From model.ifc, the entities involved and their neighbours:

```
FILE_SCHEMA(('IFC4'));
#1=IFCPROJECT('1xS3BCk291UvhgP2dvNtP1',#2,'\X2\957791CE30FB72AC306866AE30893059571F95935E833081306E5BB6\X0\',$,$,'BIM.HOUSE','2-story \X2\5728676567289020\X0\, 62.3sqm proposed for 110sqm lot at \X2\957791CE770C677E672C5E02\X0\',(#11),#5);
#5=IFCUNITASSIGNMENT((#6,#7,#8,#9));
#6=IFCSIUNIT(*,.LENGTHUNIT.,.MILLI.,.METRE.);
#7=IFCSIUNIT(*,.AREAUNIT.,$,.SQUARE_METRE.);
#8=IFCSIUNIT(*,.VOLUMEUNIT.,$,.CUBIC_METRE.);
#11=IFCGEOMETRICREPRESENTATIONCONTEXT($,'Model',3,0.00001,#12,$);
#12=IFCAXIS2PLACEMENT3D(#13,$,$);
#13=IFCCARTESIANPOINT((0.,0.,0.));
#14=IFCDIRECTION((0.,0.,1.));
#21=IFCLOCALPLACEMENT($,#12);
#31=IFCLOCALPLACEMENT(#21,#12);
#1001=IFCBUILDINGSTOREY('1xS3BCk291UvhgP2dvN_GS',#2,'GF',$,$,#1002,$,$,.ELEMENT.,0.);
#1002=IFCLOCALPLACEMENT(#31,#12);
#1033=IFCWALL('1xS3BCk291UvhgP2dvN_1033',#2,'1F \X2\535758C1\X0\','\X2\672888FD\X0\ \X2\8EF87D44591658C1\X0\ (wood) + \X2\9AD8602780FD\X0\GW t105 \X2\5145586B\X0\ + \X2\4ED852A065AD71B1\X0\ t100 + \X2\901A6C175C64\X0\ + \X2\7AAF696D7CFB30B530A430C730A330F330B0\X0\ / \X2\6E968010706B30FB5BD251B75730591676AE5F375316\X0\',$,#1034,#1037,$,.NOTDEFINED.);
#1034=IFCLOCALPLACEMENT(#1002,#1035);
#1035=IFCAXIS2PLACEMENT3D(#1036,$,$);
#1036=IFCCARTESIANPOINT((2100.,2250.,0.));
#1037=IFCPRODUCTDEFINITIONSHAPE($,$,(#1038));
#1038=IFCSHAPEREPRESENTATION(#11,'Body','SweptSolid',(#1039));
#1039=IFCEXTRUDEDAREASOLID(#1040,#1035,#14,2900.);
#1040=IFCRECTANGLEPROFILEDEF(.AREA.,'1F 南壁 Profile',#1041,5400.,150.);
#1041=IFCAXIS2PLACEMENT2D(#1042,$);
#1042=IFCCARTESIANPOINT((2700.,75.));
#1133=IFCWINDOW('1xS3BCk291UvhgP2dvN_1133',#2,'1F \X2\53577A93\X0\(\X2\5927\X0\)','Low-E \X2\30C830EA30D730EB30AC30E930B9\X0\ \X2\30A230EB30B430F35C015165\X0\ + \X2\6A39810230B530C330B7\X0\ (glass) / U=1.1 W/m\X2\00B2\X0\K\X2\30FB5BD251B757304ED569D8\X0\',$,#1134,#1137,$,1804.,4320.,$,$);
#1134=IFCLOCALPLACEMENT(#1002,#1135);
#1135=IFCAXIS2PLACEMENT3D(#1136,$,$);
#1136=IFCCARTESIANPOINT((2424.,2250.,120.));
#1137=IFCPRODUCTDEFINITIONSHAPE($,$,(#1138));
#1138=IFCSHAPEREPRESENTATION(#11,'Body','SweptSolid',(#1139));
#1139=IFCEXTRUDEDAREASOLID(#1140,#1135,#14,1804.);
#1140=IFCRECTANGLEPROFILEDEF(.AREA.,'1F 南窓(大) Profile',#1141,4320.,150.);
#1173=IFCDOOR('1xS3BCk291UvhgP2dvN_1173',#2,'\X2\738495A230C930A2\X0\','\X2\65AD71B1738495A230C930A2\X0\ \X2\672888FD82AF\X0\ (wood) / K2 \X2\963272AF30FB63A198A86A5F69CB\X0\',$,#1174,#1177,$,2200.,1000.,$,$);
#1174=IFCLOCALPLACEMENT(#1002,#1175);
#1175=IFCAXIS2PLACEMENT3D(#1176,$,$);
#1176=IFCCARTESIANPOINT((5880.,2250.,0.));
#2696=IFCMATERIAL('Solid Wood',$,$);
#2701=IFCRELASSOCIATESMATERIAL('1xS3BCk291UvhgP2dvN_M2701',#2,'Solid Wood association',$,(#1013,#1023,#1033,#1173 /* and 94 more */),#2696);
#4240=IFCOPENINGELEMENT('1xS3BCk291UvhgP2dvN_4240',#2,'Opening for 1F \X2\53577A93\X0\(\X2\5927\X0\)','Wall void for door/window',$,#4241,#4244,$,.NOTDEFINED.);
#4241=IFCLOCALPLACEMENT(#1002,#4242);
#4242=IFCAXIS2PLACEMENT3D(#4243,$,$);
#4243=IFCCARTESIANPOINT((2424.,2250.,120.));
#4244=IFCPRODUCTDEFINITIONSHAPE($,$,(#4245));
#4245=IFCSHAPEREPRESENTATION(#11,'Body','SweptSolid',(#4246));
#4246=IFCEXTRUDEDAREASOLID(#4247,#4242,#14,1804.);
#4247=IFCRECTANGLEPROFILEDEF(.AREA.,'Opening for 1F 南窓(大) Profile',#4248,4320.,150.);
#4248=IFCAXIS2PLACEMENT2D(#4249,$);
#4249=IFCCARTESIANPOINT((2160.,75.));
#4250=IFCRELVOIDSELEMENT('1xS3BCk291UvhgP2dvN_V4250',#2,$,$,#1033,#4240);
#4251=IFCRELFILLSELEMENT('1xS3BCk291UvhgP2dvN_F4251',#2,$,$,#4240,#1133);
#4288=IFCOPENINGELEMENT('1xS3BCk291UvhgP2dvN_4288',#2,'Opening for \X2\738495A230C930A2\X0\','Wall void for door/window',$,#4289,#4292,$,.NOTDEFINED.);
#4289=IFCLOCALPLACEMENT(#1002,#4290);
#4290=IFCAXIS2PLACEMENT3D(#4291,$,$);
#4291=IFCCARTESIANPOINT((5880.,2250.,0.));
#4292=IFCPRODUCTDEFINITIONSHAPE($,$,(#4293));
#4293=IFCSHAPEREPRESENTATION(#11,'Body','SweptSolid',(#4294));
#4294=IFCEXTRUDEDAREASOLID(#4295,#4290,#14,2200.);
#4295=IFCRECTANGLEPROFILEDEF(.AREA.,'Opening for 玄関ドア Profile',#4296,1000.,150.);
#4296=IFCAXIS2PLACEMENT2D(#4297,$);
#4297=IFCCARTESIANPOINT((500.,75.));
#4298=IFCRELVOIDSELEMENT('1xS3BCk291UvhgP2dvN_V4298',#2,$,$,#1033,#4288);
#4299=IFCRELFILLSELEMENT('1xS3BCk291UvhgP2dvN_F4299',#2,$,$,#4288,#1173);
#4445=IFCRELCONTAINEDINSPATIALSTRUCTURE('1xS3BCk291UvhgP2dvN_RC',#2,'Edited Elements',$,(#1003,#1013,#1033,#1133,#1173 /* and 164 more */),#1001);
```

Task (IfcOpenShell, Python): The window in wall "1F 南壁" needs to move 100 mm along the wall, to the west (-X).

```python
import ifcopenshell
import ifcopenshell.api.geometry
import ifcopenshell.util.placement
import ifcopenshell.util.unit

model = ifcopenshell.open("model.ifc")
unit_scale = ifcopenshell.util.unit.calculate_unit_scale(model)

window = model.by_guid("1xS3BCk291UvhgP2dvN_1133")
opening = window.FillsVoids[0].RelatingOpeningElement
wall = opening.VoidsElements[0].RelatingBuildingElement

wall_matrix = ifcopenshell.util.placement.get_local_placement(wall.ObjectPlacement)
shift = wall_matrix[:3, 0] * -0.1 / unit_scale
before = ifcopenshell.util.placement.get_local_placement(window.ObjectPlacement)[:3, 3].copy()

# The window is not placed relative to its opening, so move both.
for product in (opening, window):
    matrix = ifcopenshell.util.placement.get_local_placement(product.ObjectPlacement)
    matrix[:3, 3] += shift
    ifcopenshell.api.geometry.edit_object_placement(model, product=product, matrix=matrix, is_si=False)

after = ifcopenshell.util.placement.get_local_placement(window.ObjectPlacement)[:3, 3]
print("window moved by", (after - before).round(3) + 0.0)

model.write("model_rev.ifc")
```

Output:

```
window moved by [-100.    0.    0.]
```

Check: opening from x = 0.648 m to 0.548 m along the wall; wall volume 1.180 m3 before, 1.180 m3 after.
